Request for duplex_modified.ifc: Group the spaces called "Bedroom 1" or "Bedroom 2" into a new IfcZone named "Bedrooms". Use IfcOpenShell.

First a look at what the model holds.

```python
import ifcopenshell

model = ifcopenshell.open("duplex_modified.ifc")
print(model.schema)
seen = {}
for space in model.by_type("IfcSpace"):
    seen[space.LongName] = seen.get(space.LongName, 0) + 1
for name, count in sorted(seen.items(), key=str):
    print(count, "x", name)
print("zones:", [z.Name for z in model.by_type("IfcZone")][:20])
```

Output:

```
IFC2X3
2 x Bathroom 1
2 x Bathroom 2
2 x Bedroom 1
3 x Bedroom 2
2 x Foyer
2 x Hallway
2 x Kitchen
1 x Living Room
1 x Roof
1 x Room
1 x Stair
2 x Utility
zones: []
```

```python
import ifcopenshell
import ifcopenshell.api.group
import ifcopenshell.api.root

model = ifcopenshell.open("duplex_modified.ifc")

names = {"Bedroom 1", "Bedroom 2"}
spaces = [s for s in model.by_type("IfcSpace") if s.LongName in names]

zone = ifcopenshell.api.root.create_entity(model, ifc_class="IfcZone", name="Bedrooms")
ifcopenshell.api.group.assign_group(model, products=spaces, group=zone)
print(len(spaces), "spaces in", zone.Name)

model.write("duplex_modified_updated.ifc")
```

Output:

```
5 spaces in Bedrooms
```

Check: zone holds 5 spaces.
